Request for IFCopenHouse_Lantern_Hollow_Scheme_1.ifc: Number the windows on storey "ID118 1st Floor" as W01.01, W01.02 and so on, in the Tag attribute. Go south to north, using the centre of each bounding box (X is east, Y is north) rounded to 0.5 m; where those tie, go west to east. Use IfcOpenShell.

First a look at what the model holds.

```python
import ifcopenshell
import ifcopenshell.util.element
import ifcopenshell.util.placement

model = ifcopenshell.open("IFCopenHouse_Lantern_Hollow_Scheme_1.ifc")
print(model.schema)
storey = next(s for s in model.by_type("IfcBuildingStorey") if s.Name == "ID118 1st Floor")
windows = [e for e in ifcopenshell.util.element.get_decomposition(storey) if e.is_a("IfcWindow")]
for e in sorted(windows, key=lambda e: e.id()):
    origin = ifcopenshell.util.placement.get_local_placement(e.ObjectPlacement)[:3, 3]
    print(e.id(), e.Tag, e.Name, origin.round(2) + 0.0, sep=" | ")
```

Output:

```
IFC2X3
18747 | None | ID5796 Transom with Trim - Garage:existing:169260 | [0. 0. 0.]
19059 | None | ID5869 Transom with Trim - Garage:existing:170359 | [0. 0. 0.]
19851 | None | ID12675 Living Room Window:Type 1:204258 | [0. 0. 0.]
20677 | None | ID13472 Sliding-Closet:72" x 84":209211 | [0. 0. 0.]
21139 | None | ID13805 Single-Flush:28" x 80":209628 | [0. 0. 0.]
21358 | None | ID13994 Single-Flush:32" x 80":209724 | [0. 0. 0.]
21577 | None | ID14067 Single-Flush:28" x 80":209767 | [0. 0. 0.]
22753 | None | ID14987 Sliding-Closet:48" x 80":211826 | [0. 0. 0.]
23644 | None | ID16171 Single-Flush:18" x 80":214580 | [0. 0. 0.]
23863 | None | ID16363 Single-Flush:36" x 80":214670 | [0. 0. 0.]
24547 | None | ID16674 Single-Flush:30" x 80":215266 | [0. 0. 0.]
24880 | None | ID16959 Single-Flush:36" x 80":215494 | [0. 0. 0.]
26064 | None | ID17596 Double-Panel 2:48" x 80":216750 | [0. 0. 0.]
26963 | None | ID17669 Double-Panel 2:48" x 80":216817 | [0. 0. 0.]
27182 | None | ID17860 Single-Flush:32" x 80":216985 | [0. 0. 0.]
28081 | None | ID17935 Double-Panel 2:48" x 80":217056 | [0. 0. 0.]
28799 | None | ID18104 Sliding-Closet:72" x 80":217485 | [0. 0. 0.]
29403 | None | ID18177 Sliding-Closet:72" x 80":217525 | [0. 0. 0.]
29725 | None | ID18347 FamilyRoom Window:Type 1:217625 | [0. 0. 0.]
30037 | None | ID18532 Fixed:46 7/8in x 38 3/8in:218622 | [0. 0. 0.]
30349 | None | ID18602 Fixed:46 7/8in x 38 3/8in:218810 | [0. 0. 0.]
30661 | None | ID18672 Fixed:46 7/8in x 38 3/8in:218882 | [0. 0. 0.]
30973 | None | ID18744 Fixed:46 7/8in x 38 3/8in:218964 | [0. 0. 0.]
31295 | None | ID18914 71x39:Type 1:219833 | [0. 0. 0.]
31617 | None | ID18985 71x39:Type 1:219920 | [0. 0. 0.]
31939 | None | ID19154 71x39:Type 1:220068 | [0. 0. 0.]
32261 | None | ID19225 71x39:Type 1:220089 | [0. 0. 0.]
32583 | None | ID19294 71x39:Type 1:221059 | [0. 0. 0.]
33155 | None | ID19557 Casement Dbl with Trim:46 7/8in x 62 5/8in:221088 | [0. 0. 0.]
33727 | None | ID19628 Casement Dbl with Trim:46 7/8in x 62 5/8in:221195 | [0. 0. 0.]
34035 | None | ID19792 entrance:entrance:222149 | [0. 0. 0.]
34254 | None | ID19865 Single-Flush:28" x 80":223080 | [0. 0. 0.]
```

```python
import ifcopenshell
import ifcopenshell.geom
import ifcopenshell.util.element
import ifcopenshell.util.shape

model = ifcopenshell.open("IFCopenHouse_Lantern_Hollow_Scheme_1.ifc")
settings = ifcopenshell.geom.settings()
settings.set("use-world-coords", True)


def centre(element):
    shape = ifcopenshell.geom.create_shape(settings, element)
    return ifcopenshell.util.shape.get_bbox_centroid(shape.geometry)


storey = next(s for s in model.by_type("IfcBuildingStorey") if s.Name == "ID118 1st Floor")
windows = [e for e in ifcopenshell.util.element.get_decomposition(storey) if e.is_a("IfcWindow")]

# Insertion points can sit at a corner or the storey origin, so sort by the geometry (in metres).
centres = {e: centre(e) for e in windows}
windows.sort(key=lambda e: (round(centres[e][1] / 0.5), centres[e][0]))

for i, e in enumerate(windows, start=1):
    number = f"W01.{i:02d}"
    e.Tag = number
    print(e.id(), number)

model.write("IFCopenHouse_Lantern_Hollow_Scheme_1-out.ifc")
```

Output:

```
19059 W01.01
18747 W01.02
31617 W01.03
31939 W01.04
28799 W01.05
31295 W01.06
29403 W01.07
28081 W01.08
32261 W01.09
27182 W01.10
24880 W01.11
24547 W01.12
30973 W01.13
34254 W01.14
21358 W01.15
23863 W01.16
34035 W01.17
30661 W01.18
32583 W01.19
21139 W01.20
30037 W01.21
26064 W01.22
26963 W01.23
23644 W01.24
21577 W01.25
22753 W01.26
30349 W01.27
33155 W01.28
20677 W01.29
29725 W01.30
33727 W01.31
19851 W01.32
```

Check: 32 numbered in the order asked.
